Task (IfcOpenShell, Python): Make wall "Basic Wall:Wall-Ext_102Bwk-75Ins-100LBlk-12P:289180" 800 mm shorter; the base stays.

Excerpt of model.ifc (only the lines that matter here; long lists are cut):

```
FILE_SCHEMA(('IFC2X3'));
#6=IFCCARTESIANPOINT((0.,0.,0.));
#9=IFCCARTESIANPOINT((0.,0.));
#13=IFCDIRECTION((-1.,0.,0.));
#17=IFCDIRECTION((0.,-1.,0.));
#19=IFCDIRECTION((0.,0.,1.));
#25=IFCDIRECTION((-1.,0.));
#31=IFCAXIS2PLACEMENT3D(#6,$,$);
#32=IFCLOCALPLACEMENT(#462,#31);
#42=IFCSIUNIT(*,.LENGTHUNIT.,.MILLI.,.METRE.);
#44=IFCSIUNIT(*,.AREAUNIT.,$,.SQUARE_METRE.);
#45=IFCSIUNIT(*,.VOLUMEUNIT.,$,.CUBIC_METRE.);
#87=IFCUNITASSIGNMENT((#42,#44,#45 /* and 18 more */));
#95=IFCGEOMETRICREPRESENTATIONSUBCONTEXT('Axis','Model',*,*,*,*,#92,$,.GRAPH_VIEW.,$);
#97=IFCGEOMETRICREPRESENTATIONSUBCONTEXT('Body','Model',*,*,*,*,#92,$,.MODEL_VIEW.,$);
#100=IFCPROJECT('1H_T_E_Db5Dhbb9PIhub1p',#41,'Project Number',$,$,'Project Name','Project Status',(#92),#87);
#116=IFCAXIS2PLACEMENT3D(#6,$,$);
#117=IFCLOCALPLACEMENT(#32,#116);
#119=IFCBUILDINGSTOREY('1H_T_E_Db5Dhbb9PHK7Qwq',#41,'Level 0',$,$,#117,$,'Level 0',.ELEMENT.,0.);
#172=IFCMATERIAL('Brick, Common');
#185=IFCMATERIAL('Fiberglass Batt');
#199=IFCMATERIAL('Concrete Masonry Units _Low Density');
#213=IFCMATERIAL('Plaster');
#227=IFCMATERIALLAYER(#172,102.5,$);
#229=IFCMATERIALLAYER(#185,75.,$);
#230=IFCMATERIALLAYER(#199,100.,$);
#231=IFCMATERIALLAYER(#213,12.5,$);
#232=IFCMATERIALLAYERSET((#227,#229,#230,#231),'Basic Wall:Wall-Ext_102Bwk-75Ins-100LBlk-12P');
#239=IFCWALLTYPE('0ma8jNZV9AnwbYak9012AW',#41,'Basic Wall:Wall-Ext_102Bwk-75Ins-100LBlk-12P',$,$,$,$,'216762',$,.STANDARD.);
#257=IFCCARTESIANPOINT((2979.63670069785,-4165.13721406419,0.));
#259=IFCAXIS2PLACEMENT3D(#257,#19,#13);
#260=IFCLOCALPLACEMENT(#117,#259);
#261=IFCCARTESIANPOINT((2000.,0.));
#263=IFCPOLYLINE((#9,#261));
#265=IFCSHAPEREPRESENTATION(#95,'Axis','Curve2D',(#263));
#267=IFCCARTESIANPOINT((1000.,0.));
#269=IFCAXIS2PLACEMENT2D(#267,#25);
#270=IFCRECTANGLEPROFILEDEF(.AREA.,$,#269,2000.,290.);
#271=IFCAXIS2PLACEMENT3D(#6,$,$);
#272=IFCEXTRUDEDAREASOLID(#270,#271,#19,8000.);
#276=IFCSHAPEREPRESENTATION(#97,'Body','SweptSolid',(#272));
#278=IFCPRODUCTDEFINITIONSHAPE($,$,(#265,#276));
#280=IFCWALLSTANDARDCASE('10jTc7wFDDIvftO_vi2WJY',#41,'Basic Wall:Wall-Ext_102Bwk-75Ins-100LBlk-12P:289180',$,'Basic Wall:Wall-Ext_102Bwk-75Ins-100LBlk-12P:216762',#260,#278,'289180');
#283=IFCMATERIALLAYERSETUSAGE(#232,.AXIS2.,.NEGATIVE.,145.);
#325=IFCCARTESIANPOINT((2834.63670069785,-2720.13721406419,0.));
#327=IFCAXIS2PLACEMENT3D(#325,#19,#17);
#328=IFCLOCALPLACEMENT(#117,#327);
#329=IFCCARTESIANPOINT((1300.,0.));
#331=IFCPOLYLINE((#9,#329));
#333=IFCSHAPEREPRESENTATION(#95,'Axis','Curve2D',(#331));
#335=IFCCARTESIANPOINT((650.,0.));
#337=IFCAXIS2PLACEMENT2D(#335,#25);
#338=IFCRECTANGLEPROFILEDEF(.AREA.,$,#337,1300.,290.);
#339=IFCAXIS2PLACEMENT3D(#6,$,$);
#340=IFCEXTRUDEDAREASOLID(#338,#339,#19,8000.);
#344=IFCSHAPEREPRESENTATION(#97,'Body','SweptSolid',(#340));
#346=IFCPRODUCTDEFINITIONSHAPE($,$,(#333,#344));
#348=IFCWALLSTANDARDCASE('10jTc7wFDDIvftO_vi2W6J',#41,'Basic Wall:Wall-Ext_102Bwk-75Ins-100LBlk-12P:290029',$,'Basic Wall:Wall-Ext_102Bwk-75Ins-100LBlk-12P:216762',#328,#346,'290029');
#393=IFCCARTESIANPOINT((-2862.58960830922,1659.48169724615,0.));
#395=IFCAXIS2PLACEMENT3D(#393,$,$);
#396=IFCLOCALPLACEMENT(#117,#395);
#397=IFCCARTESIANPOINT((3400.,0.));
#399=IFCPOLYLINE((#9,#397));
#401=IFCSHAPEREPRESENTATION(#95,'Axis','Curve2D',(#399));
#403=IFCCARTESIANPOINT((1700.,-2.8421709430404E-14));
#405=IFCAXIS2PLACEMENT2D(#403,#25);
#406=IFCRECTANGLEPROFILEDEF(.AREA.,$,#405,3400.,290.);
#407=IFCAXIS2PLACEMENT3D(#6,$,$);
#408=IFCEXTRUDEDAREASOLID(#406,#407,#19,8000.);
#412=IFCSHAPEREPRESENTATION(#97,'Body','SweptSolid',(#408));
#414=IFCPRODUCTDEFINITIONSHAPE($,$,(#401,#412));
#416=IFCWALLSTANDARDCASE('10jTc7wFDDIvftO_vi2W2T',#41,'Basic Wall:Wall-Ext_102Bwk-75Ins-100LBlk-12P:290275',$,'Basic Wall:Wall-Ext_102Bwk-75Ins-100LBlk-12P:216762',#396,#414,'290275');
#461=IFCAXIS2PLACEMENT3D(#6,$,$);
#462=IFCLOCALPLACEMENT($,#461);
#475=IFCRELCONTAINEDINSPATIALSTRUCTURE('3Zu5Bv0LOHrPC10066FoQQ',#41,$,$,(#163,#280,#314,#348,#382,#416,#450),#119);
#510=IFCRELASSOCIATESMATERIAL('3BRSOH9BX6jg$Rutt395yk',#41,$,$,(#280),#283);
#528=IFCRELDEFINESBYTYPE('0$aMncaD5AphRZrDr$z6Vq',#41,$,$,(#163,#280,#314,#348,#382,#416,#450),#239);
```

```python
import ifcopenshell
import ifcopenshell.geom
import ifcopenshell.util.representation
import ifcopenshell.util.shape
import ifcopenshell.util.unit

model = ifcopenshell.open("model.ifc")
unit_scale = ifcopenshell.util.unit.calculate_unit_scale(model)
settings = ifcopenshell.geom.settings()


def volume(element):
    """Net volume in cubic metres, openings subtracted."""
    shape = ifcopenshell.geom.create_shape(settings, element)
    return ifcopenshell.util.shape.get_volume(shape.geometry)


wall = model.by_guid("10jTc7wFDDIvftO_vi2WJY")
before = volume(wall)

body = ifcopenshell.util.representation.get_representation(wall, "Model", "Body")
solid = body.Items[0]
old_height = solid.Depth
solid.Depth -= 0.8 / unit_scale
after = volume(wall)

print(f"height {old_height:g} -> {solid.Depth:g}, volume {before:.3f} -> {after:.3f} m3")

model.write("model-out.ifc")
```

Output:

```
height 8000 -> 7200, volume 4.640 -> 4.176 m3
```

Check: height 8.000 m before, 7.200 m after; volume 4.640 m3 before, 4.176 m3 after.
